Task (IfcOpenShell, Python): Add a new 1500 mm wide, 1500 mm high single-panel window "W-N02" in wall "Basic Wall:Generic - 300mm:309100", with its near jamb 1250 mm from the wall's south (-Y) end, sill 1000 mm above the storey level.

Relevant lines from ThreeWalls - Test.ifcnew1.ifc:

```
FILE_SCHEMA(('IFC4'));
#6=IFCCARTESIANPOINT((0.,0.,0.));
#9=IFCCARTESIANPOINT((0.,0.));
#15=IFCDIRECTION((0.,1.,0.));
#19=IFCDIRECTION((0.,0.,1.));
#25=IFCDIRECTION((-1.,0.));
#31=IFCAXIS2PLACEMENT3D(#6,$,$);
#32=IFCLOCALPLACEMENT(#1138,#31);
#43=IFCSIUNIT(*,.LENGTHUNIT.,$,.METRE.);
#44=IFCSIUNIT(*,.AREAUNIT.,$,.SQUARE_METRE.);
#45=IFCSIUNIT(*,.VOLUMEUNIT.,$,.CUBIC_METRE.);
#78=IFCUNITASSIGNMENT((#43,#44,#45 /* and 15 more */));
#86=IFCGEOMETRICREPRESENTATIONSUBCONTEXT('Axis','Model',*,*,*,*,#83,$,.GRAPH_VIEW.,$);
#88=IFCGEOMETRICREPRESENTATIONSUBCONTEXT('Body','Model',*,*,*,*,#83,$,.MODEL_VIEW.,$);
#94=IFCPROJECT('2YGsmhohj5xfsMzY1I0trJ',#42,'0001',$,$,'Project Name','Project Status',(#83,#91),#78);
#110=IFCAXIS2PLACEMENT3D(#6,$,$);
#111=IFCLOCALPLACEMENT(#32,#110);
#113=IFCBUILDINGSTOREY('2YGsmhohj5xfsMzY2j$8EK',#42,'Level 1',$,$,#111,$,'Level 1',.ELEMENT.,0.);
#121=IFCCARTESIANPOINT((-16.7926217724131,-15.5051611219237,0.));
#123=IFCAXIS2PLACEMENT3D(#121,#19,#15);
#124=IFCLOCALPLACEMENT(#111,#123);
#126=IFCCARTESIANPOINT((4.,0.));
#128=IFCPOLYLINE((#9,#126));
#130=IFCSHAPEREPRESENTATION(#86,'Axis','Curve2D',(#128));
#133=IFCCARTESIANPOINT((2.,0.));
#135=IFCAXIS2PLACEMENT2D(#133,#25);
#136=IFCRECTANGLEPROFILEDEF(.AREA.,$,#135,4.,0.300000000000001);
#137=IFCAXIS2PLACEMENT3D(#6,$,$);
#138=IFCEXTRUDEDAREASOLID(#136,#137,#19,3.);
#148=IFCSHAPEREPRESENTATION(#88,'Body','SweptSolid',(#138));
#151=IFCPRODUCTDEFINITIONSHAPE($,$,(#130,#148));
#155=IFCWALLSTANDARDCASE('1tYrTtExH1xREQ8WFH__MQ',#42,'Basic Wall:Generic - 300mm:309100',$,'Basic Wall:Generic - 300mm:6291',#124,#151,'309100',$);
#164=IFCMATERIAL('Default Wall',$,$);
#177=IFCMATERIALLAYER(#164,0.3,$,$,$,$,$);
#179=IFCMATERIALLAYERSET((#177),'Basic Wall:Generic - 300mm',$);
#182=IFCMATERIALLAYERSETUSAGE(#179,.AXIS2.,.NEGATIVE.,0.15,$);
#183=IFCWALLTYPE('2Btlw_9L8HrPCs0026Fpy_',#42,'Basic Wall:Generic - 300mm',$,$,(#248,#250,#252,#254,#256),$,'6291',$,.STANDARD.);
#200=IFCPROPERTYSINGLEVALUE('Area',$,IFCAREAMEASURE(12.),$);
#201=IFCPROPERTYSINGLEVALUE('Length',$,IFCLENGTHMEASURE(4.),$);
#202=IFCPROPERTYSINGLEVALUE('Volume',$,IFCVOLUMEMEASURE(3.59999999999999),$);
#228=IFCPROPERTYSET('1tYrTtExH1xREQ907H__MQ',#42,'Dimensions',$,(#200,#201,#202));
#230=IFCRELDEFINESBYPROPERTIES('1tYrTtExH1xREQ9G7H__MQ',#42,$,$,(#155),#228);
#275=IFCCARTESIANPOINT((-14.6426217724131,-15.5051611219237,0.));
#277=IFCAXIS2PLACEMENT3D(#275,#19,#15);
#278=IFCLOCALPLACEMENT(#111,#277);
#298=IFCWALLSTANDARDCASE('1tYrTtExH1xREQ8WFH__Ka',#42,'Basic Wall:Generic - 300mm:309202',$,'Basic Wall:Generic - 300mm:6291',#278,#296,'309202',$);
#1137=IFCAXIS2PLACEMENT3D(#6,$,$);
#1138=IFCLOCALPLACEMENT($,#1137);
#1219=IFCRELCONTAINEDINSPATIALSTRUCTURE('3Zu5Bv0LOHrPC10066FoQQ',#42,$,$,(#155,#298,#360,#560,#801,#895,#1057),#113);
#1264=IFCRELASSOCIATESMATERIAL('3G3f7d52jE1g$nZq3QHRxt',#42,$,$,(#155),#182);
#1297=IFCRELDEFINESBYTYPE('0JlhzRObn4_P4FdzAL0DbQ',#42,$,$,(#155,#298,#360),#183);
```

```python
import numpy as np
import ifcopenshell
import ifcopenshell.api.feature
import ifcopenshell.api.geometry
import ifcopenshell.api.pset
import ifcopenshell.api.root
import ifcopenshell.api.spatial
import ifcopenshell.geom
import ifcopenshell.util.element
import ifcopenshell.util.placement
import ifcopenshell.util.representation
import ifcopenshell.util.shape
import ifcopenshell.util.unit

model = ifcopenshell.open("ThreeWalls - Test.ifcnew1.ifc")
unit_scale = ifcopenshell.util.unit.calculate_unit_scale(model)
area_scale = ifcopenshell.util.unit.calculate_unit_scale(model, "AREAUNIT")
volume_scale = ifcopenshell.util.unit.calculate_unit_scale(model, "VOLUMEUNIT")
settings = ifcopenshell.geom.settings()


def volume(element):
    """Net volume in cubic metres, openings subtracted."""
    shape = ifcopenshell.geom.create_shape(settings, element)
    return ifcopenshell.util.shape.get_volume(shape.geometry)


wall = model.by_guid("1tYrTtExH1xREQ8WFH__MQ")
storey = ifcopenshell.util.element.get_container(wall, ifc_class="IfcBuildingStorey")
context = ifcopenshell.util.representation.get_context(model, "Model", "Body", "MODEL_VIEW")
before = volume(wall)

width, height, from_end, sill = 1.5, 1.5, 1.25, 1  # metres

# The wall runs along its own X axis, and the end named is its -X end.
wall_shape = ifcopenshell.geom.create_shape(settings, wall)
x, y, z = ifcopenshell.util.shape.get_vertices(wall_shape.geometry).T
start = x.min() + from_end
face, thickness = float(y.min()), float(y.max() - y.min())
wall_matrix = ifcopenshell.util.placement.get_local_placement(wall.ObjectPlacement)
level = ifcopenshell.util.placement.get_local_placement(storey.ObjectPlacement)[2, 3]


def in_wall(x, y):
    """Placement at x, y metres in the wall's axes, at sill height."""
    matrix = wall_matrix.copy()
    matrix[:, 3] = wall_matrix @ np.array([x / unit_scale, y / unit_scale, 0.0, 1.0])
    matrix[2, 3] = level + sill / unit_scale
    return matrix


# Opening: a box that overshoots both wall faces by 50 mm.
opening = ifcopenshell.api.root.create_entity(model, ifc_class="IfcOpeningElement", predefined_type="OPENING")
box = ifcopenshell.api.geometry.add_wall_representation(
    model, context=context, length=width, height=height, thickness=thickness + 0.1
)
ifcopenshell.api.geometry.assign_representation(model, product=opening, representation=box)
ifcopenshell.api.geometry.edit_object_placement(model, product=opening, matrix=in_wall(start, face - 0.05), is_si=False)
ifcopenshell.api.feature.add_feature(model, feature=opening, element=wall)

window = ifcopenshell.api.root.create_entity(model, ifc_class="IfcWindow", name="W-N02", predefined_type="WINDOW")
window.OverallWidth, window.OverallHeight = width / unit_scale, height / unit_scale
window.PartitioningType = "SINGLE_PANEL"
body = ifcopenshell.api.geometry.add_window_representation(
    model,
    context=context,
    overall_width=window.OverallWidth,
    overall_height=window.OverallHeight,
    partition_type="SINGLE_PANEL",
)
ifcopenshell.api.geometry.assign_representation(model, product=window, representation=body)
ifcopenshell.api.spatial.assign_container(model, products=[window], relating_structure=storey)
ifcopenshell.api.feature.add_filling(model, opening=opening, element=window)

# Centre the window in the wall's thickness.
ifcopenshell.api.geometry.edit_object_placement(model, product=window, matrix=in_wall(start, face), is_si=False)
window_shape = ifcopenshell.geom.create_shape(settings, window)
depth = ifcopenshell.util.shape.get_vertices(window_shape.geometry)[:, 1]
offset = face + thickness / 2 - (depth.min() + depth.max()) / 2
ifcopenshell.api.geometry.edit_object_placement(model, product=window, matrix=in_wall(start, offset), is_si=False)

after = volume(wall)

# Update the wall's stored quantities.
pset = model.by_id(ifcopenshell.util.element.get_pset(wall, "Dimensions", should_inherit=False)["id"])
ifcopenshell.api.pset.edit_pset(model, pset=pset, properties={
    "Area": model.create_entity("IfcAreaMeasure", after / thickness / area_scale),
    "Volume": model.create_entity("IfcVolumeMeasure", after / volume_scale),
})

print(f"wall volume {before:.3f} -> {after:.3f} m3")

model.write("ThreeWalls - Test.ifcnew1-out.ifc")
```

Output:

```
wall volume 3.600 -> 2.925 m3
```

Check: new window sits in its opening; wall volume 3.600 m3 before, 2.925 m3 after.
